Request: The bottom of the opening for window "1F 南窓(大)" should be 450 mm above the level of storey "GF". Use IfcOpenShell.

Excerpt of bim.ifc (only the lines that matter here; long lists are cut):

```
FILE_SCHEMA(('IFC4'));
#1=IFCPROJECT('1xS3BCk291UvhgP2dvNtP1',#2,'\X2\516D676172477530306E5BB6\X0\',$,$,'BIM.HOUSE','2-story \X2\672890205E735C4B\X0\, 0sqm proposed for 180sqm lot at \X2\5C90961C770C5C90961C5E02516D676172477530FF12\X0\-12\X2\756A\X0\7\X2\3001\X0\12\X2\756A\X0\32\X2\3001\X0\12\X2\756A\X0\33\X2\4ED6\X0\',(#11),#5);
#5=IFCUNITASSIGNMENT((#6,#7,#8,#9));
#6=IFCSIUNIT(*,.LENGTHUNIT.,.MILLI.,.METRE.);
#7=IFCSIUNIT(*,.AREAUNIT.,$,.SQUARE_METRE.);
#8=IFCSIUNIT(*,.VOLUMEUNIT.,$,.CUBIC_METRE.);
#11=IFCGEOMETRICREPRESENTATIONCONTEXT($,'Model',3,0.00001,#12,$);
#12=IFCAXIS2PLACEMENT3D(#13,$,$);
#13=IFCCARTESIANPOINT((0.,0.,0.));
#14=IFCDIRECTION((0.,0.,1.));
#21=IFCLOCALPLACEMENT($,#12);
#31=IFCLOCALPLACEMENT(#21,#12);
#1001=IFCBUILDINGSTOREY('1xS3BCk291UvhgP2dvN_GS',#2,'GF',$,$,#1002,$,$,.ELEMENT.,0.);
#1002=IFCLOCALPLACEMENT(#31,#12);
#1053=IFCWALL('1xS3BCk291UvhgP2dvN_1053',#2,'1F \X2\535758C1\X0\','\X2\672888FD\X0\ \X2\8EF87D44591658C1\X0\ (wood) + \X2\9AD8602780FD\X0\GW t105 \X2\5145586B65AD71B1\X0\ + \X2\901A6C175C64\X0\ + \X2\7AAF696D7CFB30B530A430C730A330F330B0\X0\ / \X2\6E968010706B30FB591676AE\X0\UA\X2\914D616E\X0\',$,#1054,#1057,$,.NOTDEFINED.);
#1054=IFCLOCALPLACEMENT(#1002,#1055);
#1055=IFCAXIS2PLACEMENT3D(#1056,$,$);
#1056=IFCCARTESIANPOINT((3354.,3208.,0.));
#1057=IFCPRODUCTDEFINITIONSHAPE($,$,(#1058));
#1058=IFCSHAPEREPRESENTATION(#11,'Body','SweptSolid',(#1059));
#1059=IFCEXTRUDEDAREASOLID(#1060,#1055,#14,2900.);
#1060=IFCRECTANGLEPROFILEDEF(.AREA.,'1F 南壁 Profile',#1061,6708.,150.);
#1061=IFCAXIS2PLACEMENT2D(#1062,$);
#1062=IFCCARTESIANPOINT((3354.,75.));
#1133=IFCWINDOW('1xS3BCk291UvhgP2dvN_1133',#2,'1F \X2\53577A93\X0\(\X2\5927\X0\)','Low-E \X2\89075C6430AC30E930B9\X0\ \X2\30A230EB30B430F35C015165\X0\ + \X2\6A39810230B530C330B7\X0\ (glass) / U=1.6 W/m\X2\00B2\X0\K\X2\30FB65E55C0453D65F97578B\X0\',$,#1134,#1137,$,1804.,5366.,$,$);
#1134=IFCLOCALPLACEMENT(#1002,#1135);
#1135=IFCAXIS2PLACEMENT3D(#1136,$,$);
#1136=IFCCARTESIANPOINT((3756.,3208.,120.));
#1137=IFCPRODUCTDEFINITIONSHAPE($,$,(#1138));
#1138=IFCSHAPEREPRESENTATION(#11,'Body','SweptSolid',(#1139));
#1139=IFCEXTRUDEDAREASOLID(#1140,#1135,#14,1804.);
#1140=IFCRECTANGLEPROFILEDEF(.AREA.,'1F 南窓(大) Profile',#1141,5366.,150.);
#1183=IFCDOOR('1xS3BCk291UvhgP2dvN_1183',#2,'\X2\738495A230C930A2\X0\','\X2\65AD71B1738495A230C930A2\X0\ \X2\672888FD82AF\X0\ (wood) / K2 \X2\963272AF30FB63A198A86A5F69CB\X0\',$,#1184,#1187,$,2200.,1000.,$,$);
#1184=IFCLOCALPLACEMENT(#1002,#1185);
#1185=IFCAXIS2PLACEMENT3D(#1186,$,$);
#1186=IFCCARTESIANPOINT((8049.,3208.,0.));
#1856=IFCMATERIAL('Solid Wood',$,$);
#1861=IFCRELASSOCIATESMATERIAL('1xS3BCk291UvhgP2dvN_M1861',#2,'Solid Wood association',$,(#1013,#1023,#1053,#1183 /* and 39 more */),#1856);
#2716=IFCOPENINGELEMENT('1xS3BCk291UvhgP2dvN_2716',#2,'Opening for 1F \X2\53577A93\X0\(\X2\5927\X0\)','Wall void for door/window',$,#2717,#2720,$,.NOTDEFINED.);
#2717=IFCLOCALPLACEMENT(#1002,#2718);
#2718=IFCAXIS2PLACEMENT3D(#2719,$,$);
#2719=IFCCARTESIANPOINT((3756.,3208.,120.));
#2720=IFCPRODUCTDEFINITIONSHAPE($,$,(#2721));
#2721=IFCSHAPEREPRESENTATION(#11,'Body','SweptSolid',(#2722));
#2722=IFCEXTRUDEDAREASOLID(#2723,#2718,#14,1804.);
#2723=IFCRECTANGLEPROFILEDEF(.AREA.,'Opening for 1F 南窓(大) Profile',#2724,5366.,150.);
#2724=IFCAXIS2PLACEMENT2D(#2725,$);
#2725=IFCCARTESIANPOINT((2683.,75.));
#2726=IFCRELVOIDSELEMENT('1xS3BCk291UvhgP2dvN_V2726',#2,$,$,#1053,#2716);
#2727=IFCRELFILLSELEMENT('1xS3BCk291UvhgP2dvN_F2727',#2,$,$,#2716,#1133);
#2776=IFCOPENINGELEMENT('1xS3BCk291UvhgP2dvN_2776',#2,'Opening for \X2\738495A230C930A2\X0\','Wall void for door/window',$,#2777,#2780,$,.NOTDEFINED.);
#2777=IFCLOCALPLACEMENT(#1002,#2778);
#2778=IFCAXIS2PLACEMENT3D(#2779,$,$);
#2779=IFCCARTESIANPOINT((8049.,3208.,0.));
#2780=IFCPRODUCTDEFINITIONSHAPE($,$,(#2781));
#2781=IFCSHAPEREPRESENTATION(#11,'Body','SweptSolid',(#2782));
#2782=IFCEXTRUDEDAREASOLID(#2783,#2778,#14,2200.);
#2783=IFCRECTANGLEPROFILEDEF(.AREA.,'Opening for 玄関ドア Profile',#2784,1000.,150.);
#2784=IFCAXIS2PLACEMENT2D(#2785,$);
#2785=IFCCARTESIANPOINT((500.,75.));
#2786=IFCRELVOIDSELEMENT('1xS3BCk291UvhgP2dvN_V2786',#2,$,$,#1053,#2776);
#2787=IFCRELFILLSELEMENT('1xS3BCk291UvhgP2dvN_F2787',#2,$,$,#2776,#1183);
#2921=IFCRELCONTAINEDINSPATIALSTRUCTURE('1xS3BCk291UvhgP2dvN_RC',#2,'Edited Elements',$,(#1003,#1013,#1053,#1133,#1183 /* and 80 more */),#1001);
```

```python
import numpy as np
import ifcopenshell
import ifcopenshell.api.geometry
import ifcopenshell.geom
import ifcopenshell.util.element
import ifcopenshell.util.placement
import ifcopenshell.util.shape
import ifcopenshell.util.unit

model = ifcopenshell.open("bim.ifc")
unit_scale = ifcopenshell.util.unit.calculate_unit_scale(model)

window = model.by_guid("1xS3BCk291UvhgP2dvN_1133")
opening = window.FillsVoids[0].RelatingOpeningElement
storey = ifcopenshell.util.element.get_container(window, ifc_class="IfcBuildingStorey")
level = ifcopenshell.util.placement.get_local_placement(storey.ObjectPlacement)[2, 3]

# The opening's origin need not be at the sill, so measure its lowest point.
shape = ifcopenshell.geom.create_shape(ifcopenshell.geom.settings(), opening)
bottom = ifcopenshell.util.shape.get_shape_bottom_elevation(shape, shape.geometry) / unit_scale
dz = level + 450.0 - bottom

shift = np.array([0.0, 0.0, dz])
# The window is not placed relative to its opening, so move both.
for product in (opening, window):
    matrix = ifcopenshell.util.placement.get_local_placement(product.ObjectPlacement)
    matrix[:3, 3] += shift
    ifcopenshell.api.geometry.edit_object_placement(model, product=product, matrix=matrix, is_si=False)

print(f"moved by {dz * unit_scale:+.3f} m")

model.write("bim_rev.ifc")
```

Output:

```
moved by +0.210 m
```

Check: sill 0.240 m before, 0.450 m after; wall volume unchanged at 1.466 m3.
